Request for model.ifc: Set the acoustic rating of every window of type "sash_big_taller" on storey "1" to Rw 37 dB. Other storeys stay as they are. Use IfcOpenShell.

First a look at what the model holds.

```python
import ifcopenshell
import ifcopenshell.util.element

model = ifcopenshell.open("model.ifc")
print(model.schema)
storey = next(s for s in model.by_type("IfcBuildingStorey") if s.Name == "1")
windows = [e for e in ifcopenshell.util.element.get_decomposition(storey) if e.is_a("IfcWindow")]
seen = {}
for e in windows:
    element_type = ifcopenshell.util.element.get_type(e)
    key = (element_type.Name if element_type != e and element_type else None, ifcopenshell.util.element.get_pset(e, "Pset_WindowCommon", "AcousticRating"))
    seen[key] = seen.get(key, 0) + 1
for (name, value), count in sorted(seen.items(), key=str):
    print(count, "x", name, "|", value)
```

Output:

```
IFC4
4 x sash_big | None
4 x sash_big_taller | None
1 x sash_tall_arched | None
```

```python
import ifcopenshell
import ifcopenshell.api.pset
import ifcopenshell.util.element

model = ifcopenshell.open("model.ifc")

storey = next(s for s in model.by_type("IfcBuildingStorey") if s.Name == "1")
windows = [e for e in ifcopenshell.util.element.get_decomposition(storey) if e.is_a("IfcWindow")]

count = 0
for e in windows:
    element_type = ifcopenshell.util.element.get_type(e)
    if element_type in (None, e) or element_type.Name != "sash_big_taller":
        continue
    # add_pset returns the element's existing set when there is one.
    pset = ifcopenshell.api.pset.add_pset(model, product=e, name="Pset_WindowCommon")
    ifcopenshell.api.pset.edit_pset(model, pset=pset, properties={"AcousticRating": "Rw 37 dB"})
    count += 1

print(count, "windows updated")

model.write("model-out.ifc")
```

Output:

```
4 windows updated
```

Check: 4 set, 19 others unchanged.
